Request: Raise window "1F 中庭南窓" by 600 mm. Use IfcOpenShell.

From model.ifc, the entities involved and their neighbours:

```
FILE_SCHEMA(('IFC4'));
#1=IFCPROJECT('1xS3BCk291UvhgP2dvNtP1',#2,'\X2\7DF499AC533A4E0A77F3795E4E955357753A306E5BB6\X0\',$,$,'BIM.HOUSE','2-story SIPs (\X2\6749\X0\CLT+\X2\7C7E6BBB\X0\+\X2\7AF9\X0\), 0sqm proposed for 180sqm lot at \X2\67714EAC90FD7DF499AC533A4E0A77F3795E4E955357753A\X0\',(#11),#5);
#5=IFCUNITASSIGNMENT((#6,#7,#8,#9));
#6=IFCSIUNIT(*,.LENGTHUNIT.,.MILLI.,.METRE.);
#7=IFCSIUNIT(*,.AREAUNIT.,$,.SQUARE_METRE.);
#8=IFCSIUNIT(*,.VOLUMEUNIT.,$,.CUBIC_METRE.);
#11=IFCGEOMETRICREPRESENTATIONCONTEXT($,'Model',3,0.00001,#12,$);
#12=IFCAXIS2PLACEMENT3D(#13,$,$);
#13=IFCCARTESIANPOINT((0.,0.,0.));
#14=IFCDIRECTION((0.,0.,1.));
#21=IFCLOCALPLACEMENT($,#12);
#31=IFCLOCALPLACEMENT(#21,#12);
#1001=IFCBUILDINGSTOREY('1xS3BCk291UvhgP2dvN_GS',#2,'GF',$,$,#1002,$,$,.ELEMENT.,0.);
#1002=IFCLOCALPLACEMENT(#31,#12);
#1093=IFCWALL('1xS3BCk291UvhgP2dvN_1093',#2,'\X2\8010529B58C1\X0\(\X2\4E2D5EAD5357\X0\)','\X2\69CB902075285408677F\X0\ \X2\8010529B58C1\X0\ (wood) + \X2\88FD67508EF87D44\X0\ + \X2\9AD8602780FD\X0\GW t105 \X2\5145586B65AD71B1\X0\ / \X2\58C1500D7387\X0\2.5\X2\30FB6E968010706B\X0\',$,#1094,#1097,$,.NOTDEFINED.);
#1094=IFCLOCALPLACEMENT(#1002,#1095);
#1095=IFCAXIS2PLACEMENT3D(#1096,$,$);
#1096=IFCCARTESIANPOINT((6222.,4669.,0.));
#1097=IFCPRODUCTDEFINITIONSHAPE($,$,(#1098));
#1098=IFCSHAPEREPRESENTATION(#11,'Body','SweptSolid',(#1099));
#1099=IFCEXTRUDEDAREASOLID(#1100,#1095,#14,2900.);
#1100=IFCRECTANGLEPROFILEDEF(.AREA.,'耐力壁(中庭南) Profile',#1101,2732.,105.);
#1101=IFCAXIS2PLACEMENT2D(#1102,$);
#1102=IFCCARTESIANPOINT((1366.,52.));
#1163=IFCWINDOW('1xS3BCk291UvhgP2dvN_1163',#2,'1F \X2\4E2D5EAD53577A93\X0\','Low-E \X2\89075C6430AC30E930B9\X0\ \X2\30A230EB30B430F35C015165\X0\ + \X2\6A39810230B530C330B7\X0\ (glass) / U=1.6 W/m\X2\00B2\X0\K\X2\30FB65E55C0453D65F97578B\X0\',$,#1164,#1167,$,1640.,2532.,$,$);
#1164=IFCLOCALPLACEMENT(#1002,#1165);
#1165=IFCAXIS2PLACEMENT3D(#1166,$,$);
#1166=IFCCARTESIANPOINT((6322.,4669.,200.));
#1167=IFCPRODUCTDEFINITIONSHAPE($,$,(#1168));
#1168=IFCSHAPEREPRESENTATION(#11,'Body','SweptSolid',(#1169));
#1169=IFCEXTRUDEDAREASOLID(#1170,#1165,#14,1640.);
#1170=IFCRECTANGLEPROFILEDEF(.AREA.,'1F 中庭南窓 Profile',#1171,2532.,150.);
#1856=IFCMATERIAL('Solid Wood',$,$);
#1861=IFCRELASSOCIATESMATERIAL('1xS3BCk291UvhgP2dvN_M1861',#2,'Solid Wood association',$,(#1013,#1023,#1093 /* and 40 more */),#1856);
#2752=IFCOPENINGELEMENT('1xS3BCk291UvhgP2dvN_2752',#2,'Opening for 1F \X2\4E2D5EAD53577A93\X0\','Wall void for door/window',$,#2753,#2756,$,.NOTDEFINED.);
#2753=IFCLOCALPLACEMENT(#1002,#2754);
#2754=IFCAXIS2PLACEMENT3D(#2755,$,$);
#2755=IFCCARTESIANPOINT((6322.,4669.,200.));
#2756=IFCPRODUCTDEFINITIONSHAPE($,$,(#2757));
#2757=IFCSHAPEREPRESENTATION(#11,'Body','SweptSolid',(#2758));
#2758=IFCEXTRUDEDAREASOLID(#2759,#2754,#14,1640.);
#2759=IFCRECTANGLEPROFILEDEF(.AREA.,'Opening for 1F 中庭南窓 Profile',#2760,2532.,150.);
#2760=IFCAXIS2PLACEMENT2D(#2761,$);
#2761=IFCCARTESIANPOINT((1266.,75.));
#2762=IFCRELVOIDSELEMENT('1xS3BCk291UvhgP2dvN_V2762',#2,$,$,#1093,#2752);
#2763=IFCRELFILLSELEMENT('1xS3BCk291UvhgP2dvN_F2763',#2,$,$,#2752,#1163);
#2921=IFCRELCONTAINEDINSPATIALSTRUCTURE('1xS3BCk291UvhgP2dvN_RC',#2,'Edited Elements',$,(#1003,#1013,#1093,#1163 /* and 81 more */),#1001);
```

```python
import numpy as np
import ifcopenshell
import ifcopenshell.api.geometry
import ifcopenshell.util.placement
import ifcopenshell.util.unit

model = ifcopenshell.open("model.ifc")
unit_scale = ifcopenshell.util.unit.calculate_unit_scale(model)

window = model.by_guid("1xS3BCk291UvhgP2dvN_1163")
opening = window.FillsVoids[0].RelatingOpeningElement
dz = 600.0

shift = np.array([0.0, 0.0, dz])
# The window is not placed relative to its opening, so move both.
for product in (opening, window):
    matrix = ifcopenshell.util.placement.get_local_placement(product.ObjectPlacement)
    matrix[:3, 3] += shift
    ifcopenshell.api.geometry.edit_object_placement(model, product=product, matrix=matrix, is_si=False)

print(f"moved by {dz * unit_scale:+.3f} m")

model.write("model_rev.ifc")
```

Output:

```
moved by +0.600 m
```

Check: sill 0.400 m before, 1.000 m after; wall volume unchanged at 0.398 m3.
